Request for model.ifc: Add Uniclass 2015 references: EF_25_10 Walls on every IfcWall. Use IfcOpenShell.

First a look at what the model holds.

```python
import ifcopenshell

model = ifcopenshell.open("model.ifc")
print(model.schema)
print("classifications:", [c.Name for c in model.by_type("IfcClassification")])
for ifc_class in ("IfcDoor", "IfcRoof", "IfcStair", "IfcWall", "IfcWindow"):
    print(ifc_class, len(model.by_type(ifc_class)))
```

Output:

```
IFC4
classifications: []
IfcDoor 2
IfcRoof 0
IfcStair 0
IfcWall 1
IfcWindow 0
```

```python
import ifcopenshell
import ifcopenshell.api.classification

model = ifcopenshell.open("model.ifc")

system = ifcopenshell.api.classification.add_classification(model, classification="Uniclass 2015")

codes = {
    "IfcWall": ("EF_25_10", "Walls"),
}
for ifc_class, (code, name) in codes.items():
    products = model.by_type(ifc_class)
    ifcopenshell.api.classification.add_reference(
        model, products=products, classification=system, identification=code, name=name
    )
    print(code, len(products))

model.write("model_edited.ifc")
```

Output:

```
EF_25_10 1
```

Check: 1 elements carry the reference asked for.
